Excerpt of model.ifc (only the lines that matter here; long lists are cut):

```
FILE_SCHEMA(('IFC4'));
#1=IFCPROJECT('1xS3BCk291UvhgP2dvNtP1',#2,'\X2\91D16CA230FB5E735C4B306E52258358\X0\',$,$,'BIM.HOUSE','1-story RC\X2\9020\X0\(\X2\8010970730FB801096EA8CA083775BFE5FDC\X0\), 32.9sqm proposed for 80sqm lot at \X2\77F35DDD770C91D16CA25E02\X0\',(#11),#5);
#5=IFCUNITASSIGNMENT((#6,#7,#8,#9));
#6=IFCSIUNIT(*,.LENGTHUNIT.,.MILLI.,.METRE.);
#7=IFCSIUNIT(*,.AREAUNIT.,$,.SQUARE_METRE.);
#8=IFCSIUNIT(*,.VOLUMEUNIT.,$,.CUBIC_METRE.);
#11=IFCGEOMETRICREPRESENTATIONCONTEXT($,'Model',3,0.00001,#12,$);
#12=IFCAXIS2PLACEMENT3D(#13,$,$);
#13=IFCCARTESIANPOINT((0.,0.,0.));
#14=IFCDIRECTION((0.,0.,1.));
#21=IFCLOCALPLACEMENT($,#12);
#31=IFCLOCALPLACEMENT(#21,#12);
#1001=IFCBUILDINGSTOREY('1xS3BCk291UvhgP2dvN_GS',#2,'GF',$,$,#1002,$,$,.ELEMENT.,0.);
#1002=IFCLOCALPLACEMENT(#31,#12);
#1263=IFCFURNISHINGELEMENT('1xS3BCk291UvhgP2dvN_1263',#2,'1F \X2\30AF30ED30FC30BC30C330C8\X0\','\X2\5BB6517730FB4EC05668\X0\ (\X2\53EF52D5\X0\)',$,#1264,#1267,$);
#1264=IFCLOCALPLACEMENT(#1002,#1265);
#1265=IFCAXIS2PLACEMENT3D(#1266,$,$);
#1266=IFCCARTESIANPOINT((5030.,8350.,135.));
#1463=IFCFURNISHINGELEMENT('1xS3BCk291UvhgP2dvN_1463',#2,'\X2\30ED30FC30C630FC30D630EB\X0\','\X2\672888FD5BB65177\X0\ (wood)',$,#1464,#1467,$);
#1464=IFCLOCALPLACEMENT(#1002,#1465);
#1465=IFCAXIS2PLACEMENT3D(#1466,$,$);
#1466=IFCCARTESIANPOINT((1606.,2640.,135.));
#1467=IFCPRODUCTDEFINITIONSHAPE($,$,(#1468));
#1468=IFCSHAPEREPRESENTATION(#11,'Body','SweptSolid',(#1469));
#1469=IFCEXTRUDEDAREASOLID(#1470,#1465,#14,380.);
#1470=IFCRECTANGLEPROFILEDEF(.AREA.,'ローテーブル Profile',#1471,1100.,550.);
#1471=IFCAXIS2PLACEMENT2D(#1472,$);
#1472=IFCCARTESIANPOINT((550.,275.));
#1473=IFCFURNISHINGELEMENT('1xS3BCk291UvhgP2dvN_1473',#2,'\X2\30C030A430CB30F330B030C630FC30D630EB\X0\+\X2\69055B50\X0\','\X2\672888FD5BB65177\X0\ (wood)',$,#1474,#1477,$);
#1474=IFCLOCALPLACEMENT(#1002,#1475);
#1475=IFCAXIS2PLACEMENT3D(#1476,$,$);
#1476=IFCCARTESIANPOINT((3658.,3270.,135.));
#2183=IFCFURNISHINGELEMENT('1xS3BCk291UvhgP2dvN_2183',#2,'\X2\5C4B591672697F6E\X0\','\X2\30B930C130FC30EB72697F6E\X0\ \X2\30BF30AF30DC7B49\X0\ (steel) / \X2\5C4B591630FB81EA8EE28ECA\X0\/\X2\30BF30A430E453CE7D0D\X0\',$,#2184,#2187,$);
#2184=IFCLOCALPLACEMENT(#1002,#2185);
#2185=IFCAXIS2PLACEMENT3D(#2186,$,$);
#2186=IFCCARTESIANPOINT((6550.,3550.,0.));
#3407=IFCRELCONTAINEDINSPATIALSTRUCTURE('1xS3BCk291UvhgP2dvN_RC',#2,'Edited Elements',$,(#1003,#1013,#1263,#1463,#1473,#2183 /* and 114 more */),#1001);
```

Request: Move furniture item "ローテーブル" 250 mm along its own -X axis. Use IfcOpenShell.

```python
import ifcopenshell
import ifcopenshell.api.geometry
import ifcopenshell.util.placement
import ifcopenshell.util.unit

model = ifcopenshell.open("model.ifc")
unit_scale = ifcopenshell.util.unit.calculate_unit_scale(model)

item = model.by_guid("1xS3BCk291UvhgP2dvN_1463")
matrix = ifcopenshell.util.placement.get_local_placement(item.ObjectPlacement)
matrix[:3, 3] -= matrix[:3, 0] * 0.25 / unit_scale
ifcopenshell.api.geometry.edit_object_placement(model, product=item, matrix=matrix, is_si=False)

print(ifcopenshell.util.placement.get_local_placement(item.ObjectPlacement).round(3) + 0.0)

model.write("model-out.ifc")
```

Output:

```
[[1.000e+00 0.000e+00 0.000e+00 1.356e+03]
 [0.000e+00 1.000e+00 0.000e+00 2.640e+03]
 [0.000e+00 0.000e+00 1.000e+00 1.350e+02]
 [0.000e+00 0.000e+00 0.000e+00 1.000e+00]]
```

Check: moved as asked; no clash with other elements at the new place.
